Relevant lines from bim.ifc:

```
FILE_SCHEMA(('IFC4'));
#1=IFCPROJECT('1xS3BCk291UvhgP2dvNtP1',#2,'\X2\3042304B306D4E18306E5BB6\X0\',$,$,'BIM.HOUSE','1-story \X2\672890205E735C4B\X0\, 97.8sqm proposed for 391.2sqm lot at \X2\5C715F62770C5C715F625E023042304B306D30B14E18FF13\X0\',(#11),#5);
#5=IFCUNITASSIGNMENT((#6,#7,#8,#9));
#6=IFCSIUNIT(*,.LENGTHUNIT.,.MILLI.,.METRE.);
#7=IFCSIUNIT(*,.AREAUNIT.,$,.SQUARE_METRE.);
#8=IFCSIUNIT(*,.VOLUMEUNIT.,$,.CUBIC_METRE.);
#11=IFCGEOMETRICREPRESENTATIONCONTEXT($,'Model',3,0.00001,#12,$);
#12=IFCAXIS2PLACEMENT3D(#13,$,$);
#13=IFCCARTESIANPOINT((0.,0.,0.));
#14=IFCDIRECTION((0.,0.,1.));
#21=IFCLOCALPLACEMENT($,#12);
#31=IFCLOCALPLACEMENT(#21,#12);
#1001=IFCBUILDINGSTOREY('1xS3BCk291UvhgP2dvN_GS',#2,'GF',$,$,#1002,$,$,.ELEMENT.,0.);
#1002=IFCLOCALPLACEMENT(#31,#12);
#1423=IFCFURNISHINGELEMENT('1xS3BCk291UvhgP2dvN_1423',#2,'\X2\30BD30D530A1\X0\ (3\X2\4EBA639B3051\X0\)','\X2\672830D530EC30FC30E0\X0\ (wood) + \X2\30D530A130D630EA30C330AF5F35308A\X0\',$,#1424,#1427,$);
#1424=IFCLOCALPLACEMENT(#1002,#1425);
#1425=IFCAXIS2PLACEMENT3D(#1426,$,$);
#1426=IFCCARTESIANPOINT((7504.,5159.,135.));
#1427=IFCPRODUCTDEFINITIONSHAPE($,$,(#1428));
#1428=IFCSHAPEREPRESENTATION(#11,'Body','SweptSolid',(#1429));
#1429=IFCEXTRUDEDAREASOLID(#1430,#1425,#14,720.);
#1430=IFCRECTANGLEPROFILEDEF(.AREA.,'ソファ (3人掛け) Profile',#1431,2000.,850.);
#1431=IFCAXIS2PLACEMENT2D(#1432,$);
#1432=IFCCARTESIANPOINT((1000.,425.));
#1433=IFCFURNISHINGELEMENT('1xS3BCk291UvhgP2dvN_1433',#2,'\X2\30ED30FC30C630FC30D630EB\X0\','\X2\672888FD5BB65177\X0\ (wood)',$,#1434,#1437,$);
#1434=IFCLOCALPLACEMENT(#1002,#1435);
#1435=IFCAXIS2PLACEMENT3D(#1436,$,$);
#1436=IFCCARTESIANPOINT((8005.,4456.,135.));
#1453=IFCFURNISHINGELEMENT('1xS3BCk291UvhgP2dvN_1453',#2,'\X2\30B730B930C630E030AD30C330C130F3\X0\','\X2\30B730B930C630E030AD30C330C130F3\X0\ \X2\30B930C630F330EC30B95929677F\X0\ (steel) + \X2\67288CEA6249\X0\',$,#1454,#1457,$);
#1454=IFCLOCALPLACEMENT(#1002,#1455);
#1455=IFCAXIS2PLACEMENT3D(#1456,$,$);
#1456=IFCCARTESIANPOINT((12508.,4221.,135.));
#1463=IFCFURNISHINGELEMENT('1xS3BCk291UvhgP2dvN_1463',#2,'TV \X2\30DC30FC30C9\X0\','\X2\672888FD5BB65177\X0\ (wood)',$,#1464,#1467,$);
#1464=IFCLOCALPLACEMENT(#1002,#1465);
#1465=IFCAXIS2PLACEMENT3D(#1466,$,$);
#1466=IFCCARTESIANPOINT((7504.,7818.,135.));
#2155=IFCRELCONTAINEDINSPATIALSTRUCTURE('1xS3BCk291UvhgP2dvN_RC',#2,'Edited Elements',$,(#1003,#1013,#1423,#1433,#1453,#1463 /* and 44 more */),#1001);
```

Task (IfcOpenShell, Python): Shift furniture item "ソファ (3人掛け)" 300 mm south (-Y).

```python
import ifcopenshell
import ifcopenshell.api.geometry
import ifcopenshell.util.placement
import ifcopenshell.util.unit

model = ifcopenshell.open("bim.ifc")
unit_scale = ifcopenshell.util.unit.calculate_unit_scale(model)

item = model.by_id(1423)
matrix = ifcopenshell.util.placement.get_local_placement(item.ObjectPlacement)
matrix[1, 3] -= 0.3 / unit_scale
ifcopenshell.api.geometry.edit_object_placement(model, product=item, matrix=matrix, is_si=False)

print(ifcopenshell.util.placement.get_local_placement(item.ObjectPlacement).round(3) + 0.0)

model.write("bim_edited.ifc")
```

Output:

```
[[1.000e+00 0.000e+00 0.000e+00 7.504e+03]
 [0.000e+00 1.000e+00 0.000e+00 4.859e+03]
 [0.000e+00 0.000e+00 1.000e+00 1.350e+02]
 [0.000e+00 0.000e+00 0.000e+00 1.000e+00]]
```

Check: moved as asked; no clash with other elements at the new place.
